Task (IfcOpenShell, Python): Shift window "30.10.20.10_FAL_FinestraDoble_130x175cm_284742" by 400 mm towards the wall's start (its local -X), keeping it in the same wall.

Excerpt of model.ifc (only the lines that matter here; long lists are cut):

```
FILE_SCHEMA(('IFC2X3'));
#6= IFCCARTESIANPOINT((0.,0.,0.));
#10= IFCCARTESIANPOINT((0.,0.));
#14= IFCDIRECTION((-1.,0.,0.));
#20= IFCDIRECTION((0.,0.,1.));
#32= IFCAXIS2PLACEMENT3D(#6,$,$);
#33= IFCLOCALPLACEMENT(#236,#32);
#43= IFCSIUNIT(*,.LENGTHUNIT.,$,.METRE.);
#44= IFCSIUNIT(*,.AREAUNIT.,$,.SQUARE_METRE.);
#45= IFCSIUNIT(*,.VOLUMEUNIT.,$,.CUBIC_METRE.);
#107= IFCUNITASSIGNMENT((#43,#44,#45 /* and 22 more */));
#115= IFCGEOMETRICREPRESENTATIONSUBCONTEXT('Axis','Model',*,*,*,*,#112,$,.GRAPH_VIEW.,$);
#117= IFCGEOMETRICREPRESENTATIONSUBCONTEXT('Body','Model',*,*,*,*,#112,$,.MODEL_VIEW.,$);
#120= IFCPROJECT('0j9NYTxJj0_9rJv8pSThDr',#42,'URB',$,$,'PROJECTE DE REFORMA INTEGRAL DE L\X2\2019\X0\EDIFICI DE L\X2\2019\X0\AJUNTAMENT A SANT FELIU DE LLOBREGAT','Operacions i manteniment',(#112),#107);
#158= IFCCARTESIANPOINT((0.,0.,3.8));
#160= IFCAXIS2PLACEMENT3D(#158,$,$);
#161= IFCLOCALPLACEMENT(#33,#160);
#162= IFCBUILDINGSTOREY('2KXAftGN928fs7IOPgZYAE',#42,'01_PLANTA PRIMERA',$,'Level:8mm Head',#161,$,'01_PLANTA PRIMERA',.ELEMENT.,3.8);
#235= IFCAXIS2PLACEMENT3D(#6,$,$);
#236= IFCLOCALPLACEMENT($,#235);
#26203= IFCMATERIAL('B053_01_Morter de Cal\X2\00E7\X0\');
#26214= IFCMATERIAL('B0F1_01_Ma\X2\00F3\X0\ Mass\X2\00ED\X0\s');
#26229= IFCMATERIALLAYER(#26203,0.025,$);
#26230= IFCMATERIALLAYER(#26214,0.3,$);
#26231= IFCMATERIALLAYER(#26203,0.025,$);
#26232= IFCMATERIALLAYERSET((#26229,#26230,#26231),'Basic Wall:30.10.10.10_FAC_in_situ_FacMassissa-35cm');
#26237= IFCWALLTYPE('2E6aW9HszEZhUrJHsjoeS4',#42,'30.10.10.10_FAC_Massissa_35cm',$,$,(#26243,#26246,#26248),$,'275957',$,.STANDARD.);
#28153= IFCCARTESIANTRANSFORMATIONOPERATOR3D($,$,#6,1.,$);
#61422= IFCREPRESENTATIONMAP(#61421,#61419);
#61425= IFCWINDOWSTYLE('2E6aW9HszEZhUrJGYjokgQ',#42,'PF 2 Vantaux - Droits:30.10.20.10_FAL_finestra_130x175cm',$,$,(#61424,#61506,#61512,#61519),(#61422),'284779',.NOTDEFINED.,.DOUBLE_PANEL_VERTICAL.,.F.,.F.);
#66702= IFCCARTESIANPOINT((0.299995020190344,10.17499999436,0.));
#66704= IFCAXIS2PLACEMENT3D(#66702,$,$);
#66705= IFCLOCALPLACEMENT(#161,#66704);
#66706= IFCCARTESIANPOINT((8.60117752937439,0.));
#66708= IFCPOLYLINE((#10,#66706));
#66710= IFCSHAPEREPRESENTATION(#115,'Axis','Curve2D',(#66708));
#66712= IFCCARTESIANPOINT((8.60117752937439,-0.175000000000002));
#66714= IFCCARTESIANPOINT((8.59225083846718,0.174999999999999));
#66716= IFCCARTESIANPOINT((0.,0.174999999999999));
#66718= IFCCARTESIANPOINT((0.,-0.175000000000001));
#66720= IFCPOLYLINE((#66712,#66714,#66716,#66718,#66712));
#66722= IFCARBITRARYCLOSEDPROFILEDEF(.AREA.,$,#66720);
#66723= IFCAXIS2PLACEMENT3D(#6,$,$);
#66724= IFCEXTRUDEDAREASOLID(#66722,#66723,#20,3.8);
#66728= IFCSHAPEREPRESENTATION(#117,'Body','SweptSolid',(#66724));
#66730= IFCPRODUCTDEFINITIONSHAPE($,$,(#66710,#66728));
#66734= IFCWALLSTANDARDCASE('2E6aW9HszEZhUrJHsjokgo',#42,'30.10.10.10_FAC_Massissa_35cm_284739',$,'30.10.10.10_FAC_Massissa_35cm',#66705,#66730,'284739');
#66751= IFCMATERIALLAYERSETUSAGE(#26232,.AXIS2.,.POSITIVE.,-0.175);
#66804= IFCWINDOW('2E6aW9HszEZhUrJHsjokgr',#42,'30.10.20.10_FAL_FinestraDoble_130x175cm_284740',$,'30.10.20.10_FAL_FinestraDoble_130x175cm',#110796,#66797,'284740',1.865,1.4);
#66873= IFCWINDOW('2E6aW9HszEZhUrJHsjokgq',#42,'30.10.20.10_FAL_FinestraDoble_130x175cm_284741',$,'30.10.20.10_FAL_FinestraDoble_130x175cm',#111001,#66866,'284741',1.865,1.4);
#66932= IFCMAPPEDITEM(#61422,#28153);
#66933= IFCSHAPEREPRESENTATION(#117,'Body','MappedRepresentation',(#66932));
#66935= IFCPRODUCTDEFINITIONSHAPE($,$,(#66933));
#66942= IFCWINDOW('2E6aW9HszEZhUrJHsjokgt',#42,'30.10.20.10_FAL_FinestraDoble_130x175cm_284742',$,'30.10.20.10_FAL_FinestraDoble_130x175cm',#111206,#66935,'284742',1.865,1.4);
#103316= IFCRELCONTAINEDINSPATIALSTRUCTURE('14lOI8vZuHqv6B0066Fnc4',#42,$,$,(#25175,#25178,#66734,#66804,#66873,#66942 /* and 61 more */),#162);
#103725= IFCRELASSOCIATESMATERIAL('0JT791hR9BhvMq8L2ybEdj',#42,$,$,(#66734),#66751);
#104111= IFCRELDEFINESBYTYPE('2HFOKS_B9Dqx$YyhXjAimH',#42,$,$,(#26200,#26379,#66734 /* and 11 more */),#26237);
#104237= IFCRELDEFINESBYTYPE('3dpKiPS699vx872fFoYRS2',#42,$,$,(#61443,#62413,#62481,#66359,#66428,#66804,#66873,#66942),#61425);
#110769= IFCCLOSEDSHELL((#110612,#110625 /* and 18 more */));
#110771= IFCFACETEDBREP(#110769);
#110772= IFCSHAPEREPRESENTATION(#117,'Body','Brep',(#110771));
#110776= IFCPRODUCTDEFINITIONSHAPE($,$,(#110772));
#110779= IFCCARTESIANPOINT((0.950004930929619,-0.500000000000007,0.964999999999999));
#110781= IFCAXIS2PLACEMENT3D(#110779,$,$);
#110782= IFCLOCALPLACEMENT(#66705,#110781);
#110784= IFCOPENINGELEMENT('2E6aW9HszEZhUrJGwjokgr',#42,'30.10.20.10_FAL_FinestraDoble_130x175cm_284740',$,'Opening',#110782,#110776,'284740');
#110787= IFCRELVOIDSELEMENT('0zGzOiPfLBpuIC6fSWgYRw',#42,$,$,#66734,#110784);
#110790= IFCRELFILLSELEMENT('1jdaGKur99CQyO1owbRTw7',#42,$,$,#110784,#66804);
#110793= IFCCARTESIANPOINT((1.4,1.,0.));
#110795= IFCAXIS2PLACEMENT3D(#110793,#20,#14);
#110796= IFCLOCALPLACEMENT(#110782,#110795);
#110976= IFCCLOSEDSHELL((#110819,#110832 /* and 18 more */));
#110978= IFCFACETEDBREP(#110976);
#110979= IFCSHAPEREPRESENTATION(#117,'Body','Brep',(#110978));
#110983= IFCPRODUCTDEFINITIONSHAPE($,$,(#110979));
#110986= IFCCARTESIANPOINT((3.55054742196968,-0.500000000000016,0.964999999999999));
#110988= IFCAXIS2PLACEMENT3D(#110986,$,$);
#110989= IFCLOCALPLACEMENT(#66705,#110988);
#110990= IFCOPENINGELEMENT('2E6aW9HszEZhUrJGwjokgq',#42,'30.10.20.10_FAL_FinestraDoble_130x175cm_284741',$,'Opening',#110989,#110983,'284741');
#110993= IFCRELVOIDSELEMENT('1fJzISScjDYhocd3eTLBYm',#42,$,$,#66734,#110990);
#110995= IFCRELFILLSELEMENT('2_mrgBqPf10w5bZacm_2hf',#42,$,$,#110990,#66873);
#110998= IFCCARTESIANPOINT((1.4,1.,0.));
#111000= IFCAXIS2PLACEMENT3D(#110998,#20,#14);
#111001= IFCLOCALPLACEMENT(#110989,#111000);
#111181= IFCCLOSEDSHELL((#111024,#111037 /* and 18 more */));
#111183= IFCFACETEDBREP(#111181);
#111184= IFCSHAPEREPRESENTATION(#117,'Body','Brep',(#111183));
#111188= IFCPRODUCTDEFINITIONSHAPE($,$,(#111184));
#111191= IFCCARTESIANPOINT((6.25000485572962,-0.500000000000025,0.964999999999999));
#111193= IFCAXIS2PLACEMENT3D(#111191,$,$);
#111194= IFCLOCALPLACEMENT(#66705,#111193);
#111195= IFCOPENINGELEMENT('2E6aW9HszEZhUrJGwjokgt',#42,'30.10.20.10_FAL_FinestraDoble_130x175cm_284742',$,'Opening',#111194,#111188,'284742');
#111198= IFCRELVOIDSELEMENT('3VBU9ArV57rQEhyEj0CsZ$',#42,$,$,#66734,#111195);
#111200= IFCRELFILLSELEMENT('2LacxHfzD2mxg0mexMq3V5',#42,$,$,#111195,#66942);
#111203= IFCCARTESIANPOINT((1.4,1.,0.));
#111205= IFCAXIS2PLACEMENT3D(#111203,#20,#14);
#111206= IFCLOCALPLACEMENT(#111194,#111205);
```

```python
import ifcopenshell
import ifcopenshell.api.geometry
import ifcopenshell.util.placement

model = ifcopenshell.open("model.ifc")

window = model.by_guid("2E6aW9HszEZhUrJHsjokgt")
opening = window.FillsVoids[0].RelatingOpeningElement
wall = opening.VoidsElements[0].RelatingBuildingElement

wall_matrix = ifcopenshell.util.placement.get_local_placement(wall.ObjectPlacement)
shift = wall_matrix[:3, 0] * -0.4
before = ifcopenshell.util.placement.get_local_placement(window.ObjectPlacement)[:3, 3].copy()

# The window is placed relative to its opening, so it follows when the opening moves.
matrix = ifcopenshell.util.placement.get_local_placement(opening.ObjectPlacement)
matrix[:3, 3] += shift
ifcopenshell.api.geometry.edit_object_placement(
    model, product=opening, matrix=matrix, is_si=False, should_transform_children=True
)

after = ifcopenshell.util.placement.get_local_placement(window.ObjectPlacement)[:3, 3]
print("window moved by", (after - before).round(3) + 0.0)

model.write("model-out.ifc")
```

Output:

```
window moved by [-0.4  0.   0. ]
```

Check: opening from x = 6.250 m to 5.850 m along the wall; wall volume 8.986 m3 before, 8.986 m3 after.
